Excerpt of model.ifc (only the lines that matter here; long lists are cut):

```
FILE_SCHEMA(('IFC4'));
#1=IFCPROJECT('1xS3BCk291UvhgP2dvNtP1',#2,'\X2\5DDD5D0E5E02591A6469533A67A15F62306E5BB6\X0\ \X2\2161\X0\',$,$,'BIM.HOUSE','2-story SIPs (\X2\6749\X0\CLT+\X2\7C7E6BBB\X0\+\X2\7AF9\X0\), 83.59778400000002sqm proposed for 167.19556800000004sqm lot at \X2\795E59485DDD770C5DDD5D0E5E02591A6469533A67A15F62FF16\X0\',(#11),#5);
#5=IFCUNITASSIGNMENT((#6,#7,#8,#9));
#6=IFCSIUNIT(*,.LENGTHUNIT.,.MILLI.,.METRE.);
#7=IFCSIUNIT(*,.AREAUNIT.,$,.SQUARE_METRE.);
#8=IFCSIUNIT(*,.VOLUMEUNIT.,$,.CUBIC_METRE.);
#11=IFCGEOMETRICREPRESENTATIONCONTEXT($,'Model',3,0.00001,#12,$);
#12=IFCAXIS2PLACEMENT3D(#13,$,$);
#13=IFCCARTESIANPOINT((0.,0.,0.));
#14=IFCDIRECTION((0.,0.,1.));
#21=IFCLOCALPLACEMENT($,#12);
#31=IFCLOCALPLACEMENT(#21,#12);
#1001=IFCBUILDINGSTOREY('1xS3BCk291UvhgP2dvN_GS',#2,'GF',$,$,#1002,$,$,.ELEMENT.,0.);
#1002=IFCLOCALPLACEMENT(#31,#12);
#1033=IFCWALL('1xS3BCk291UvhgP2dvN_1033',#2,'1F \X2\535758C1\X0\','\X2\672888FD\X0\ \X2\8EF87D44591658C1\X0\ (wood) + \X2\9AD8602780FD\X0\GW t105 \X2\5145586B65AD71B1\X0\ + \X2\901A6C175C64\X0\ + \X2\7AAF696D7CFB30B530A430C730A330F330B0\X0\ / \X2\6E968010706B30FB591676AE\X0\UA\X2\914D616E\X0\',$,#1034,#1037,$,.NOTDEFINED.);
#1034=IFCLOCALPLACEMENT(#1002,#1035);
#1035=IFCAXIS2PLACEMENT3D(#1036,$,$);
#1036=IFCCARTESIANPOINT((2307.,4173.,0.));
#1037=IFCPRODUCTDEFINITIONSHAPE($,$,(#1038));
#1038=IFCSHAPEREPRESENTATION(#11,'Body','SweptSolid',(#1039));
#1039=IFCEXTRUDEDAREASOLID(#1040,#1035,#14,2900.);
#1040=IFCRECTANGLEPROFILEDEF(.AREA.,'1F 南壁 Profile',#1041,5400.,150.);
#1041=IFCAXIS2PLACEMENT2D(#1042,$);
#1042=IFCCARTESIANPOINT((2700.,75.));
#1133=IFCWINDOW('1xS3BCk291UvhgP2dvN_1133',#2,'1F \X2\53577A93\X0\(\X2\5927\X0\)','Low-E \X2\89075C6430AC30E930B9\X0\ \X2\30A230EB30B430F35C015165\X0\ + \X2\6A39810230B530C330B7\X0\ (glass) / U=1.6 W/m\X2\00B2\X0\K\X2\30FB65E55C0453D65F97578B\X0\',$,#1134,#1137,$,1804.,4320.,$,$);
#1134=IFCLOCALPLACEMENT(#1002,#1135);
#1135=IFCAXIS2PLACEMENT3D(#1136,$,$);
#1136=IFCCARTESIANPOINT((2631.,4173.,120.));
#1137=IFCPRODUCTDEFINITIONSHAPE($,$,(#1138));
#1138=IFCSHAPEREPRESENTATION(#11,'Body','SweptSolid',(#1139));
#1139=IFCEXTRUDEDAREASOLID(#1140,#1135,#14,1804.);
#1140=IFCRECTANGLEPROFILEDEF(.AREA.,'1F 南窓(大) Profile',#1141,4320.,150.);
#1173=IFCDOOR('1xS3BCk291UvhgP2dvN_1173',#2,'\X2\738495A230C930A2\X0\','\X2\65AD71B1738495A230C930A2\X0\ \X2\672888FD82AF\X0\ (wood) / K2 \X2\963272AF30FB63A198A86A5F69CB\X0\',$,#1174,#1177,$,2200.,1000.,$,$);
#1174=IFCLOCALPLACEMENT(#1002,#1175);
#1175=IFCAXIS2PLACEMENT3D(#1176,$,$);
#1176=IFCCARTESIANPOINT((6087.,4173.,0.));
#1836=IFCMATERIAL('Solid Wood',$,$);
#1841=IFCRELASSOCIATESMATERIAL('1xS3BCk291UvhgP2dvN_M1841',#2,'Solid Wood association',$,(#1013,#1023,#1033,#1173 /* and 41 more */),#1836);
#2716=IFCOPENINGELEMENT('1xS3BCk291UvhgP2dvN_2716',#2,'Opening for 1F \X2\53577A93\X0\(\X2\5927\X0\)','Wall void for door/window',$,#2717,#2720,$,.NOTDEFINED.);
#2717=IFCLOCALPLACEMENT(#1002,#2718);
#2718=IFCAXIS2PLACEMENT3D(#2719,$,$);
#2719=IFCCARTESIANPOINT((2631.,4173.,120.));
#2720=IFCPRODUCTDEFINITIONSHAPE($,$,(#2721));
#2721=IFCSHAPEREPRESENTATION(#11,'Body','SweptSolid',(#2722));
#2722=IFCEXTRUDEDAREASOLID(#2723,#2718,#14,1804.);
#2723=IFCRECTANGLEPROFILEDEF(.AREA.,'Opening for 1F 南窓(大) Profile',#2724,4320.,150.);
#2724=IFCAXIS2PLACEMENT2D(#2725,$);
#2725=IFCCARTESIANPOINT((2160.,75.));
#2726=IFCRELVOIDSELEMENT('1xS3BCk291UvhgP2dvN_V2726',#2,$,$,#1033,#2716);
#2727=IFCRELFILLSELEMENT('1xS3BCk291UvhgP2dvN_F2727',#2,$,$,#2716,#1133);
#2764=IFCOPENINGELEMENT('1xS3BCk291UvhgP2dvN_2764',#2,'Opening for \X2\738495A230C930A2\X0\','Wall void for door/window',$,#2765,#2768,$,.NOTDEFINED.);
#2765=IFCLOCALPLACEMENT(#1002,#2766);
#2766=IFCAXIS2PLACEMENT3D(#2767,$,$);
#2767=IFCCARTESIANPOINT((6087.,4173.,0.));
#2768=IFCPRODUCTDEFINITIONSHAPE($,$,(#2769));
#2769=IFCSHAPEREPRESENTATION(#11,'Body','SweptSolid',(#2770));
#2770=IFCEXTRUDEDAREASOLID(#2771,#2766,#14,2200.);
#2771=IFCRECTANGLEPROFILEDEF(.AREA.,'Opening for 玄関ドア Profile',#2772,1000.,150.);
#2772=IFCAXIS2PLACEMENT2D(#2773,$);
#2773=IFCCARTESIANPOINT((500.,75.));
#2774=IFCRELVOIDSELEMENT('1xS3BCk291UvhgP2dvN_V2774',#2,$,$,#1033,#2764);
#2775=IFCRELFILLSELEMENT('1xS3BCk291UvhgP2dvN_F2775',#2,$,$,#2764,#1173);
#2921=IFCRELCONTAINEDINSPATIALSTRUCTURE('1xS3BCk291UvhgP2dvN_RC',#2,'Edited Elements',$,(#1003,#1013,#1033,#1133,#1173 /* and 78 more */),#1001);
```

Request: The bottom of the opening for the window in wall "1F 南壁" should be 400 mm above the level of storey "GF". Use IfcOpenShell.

```python
import numpy as np
import ifcopenshell
import ifcopenshell.api.geometry
import ifcopenshell.geom
import ifcopenshell.util.element
import ifcopenshell.util.placement
import ifcopenshell.util.shape
import ifcopenshell.util.unit

model = ifcopenshell.open("model.ifc")
unit_scale = ifcopenshell.util.unit.calculate_unit_scale(model)

window = model.by_guid("1xS3BCk291UvhgP2dvN_1133")
opening = window.FillsVoids[0].RelatingOpeningElement
storey = ifcopenshell.util.element.get_container(window, ifc_class="IfcBuildingStorey")
level = ifcopenshell.util.placement.get_local_placement(storey.ObjectPlacement)[2, 3]

# The opening's origin need not be at the sill, so measure its lowest point.
shape = ifcopenshell.geom.create_shape(ifcopenshell.geom.settings(), opening)
bottom = ifcopenshell.util.shape.get_shape_bottom_elevation(shape, shape.geometry) / unit_scale
dz = level + 400.0 - bottom

shift = np.array([0.0, 0.0, dz])
# The window is not placed relative to its opening, so move both.
for product in (opening, window):
    matrix = ifcopenshell.util.placement.get_local_placement(product.ObjectPlacement)
    matrix[:3, 3] += shift
    ifcopenshell.api.geometry.edit_object_placement(model, product=product, matrix=matrix, is_si=False)

print(f"moved by {dz * unit_scale:+.3f} m")

model.write("model_rev.ifc")
```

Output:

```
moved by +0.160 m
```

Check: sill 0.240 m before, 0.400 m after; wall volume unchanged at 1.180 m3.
